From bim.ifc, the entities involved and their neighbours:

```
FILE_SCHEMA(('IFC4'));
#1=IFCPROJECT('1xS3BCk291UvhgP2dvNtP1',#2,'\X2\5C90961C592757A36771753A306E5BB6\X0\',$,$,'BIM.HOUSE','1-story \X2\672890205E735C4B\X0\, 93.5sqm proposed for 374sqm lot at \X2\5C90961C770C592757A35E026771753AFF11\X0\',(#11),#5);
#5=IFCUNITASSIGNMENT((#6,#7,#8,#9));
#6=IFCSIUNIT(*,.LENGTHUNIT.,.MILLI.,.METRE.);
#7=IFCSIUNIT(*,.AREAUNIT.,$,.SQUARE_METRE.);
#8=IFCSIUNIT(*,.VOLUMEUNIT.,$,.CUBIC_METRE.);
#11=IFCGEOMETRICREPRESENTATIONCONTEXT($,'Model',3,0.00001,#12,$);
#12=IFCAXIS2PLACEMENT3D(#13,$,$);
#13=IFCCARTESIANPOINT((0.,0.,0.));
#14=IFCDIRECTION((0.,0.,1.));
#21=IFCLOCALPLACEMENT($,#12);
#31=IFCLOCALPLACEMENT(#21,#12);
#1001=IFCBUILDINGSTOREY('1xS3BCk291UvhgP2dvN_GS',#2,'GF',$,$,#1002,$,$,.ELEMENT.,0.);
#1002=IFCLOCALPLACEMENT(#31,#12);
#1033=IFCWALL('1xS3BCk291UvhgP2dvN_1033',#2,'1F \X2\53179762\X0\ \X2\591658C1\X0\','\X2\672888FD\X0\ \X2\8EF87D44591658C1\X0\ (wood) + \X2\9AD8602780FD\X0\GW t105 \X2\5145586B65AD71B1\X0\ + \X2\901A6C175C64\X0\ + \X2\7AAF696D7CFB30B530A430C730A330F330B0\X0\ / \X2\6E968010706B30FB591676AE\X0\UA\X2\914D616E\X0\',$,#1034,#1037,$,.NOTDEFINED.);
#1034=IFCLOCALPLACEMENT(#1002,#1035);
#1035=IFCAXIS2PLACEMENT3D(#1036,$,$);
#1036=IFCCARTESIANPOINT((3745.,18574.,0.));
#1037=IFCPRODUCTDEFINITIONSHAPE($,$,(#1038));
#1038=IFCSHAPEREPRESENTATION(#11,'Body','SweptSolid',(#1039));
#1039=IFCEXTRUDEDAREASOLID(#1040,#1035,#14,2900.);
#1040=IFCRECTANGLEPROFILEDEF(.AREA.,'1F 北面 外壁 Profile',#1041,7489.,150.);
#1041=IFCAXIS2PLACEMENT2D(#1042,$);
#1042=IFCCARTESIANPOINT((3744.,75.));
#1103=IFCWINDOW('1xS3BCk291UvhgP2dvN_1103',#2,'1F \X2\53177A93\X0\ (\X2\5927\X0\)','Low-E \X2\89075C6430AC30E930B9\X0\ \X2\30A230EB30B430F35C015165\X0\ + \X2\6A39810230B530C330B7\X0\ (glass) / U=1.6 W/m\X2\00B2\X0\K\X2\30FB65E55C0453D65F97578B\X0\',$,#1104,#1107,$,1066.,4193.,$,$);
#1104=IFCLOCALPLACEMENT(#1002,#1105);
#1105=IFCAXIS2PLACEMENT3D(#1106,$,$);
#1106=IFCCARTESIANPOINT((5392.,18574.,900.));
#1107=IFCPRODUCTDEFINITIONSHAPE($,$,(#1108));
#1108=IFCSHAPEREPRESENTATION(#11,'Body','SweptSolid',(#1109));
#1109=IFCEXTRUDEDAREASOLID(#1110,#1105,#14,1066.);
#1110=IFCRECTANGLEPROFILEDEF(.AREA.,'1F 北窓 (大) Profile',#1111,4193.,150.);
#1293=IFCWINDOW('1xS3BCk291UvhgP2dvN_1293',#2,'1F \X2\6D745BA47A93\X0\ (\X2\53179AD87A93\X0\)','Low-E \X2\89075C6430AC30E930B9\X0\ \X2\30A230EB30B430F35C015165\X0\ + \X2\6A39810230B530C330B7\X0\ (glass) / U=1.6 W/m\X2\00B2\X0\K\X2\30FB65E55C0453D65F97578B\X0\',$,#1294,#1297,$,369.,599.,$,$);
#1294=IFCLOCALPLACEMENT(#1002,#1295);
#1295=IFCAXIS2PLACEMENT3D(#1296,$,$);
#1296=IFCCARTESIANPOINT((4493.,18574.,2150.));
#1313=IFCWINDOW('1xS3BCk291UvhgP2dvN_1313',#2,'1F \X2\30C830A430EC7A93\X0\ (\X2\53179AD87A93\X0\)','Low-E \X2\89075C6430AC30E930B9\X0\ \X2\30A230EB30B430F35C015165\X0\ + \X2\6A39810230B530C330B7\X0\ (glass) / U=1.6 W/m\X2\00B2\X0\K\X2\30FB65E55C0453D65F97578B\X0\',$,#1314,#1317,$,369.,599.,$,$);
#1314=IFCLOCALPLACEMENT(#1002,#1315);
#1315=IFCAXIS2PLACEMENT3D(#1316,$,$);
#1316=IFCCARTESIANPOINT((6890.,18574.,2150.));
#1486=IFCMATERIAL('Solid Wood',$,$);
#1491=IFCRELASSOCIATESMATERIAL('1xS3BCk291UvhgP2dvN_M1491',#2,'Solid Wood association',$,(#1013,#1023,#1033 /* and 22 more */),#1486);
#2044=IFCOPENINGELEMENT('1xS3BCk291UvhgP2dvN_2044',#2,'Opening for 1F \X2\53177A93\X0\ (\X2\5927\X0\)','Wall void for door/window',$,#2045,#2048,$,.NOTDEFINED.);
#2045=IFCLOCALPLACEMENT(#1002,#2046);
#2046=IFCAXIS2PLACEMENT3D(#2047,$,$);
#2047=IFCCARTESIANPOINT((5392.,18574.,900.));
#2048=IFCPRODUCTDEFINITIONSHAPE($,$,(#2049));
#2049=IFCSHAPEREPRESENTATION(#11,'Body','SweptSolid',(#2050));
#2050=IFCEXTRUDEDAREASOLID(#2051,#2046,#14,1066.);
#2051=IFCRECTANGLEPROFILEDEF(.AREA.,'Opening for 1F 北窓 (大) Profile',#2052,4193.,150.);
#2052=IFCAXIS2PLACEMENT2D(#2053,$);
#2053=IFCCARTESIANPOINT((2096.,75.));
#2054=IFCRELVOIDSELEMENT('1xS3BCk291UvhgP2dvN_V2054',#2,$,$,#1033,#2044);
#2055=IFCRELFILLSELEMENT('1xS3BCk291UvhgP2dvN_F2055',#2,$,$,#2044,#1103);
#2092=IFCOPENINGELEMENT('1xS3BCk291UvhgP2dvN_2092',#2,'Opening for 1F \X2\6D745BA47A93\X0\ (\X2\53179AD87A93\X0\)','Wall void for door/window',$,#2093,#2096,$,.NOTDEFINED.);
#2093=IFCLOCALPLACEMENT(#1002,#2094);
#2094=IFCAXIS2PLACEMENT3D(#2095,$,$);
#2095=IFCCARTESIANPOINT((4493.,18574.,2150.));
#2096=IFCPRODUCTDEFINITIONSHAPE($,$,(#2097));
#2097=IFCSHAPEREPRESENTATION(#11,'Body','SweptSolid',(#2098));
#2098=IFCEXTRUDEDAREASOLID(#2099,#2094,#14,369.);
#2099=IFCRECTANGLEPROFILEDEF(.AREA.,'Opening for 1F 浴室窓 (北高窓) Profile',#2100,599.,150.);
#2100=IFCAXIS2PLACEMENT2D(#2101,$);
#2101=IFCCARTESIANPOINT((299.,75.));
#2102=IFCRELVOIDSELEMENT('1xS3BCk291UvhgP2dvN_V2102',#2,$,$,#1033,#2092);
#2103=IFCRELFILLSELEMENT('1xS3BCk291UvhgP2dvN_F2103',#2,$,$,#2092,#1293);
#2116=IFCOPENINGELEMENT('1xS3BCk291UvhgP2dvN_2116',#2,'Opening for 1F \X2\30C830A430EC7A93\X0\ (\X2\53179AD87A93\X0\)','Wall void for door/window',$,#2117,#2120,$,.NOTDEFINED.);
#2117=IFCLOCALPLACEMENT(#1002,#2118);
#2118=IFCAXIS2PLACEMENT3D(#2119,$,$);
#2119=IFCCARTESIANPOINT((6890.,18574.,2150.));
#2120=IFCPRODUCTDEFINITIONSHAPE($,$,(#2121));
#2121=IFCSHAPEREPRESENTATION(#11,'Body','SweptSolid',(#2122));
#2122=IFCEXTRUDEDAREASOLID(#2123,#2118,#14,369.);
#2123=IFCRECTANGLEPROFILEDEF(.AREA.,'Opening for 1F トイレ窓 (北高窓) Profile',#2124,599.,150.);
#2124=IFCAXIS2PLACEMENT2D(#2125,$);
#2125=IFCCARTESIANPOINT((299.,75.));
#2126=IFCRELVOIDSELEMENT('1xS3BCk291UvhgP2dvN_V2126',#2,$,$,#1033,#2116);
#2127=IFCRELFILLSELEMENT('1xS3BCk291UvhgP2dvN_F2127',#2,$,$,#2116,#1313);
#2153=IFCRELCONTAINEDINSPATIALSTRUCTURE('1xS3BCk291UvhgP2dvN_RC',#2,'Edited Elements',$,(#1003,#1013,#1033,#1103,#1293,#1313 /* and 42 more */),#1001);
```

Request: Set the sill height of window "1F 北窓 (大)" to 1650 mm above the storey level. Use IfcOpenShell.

```python
import numpy as np
import ifcopenshell
import ifcopenshell.api.geometry
import ifcopenshell.geom
import ifcopenshell.util.element
import ifcopenshell.util.placement
import ifcopenshell.util.shape
import ifcopenshell.util.unit

model = ifcopenshell.open("bim.ifc")
unit_scale = ifcopenshell.util.unit.calculate_unit_scale(model)

window = model.by_id(1103)
opening = window.FillsVoids[0].RelatingOpeningElement
storey = ifcopenshell.util.element.get_container(window, ifc_class="IfcBuildingStorey")
level = ifcopenshell.util.placement.get_local_placement(storey.ObjectPlacement)[2, 3]

# The opening's origin need not be at the sill, so measure its lowest point.
shape = ifcopenshell.geom.create_shape(ifcopenshell.geom.settings(), opening)
bottom = ifcopenshell.util.shape.get_shape_bottom_elevation(shape, shape.geometry) / unit_scale
dz = level + 1.65 / unit_scale - bottom

shift = np.array([0.0, 0.0, dz])
# The window is not placed relative to its opening, so move both.
for product in (opening, window):
    matrix = ifcopenshell.util.placement.get_local_placement(product.ObjectPlacement)
    matrix[:3, 3] += shift
    ifcopenshell.api.geometry.edit_object_placement(model, product=product, matrix=matrix, is_si=False)

print(f"moved by {dz * unit_scale:+.3f} m")

model.write("bim-out.ifc")
```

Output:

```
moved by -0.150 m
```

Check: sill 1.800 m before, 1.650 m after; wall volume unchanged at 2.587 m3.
